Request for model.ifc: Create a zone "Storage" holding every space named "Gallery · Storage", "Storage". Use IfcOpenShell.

First a look at what the model holds.

```python
import ifcopenshell

model = ifcopenshell.open("model.ifc")
print(model.schema)
seen = {}
for space in model.by_type("IfcSpace"):
    seen[space.Name] = seen.get(space.Name, 0) + 1
for name, count in sorted(seen.items(), key=str):
    print(count, "x", name)
print("zones:", [z.Name for z in model.by_type("IfcZone")][:20])
```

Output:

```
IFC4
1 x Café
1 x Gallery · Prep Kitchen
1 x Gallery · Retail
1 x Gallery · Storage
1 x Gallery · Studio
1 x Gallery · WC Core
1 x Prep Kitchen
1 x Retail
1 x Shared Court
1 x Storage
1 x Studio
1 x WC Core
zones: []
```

```python
import ifcopenshell
import ifcopenshell.api.group
import ifcopenshell.api.root

model = ifcopenshell.open("model.ifc")

names = {"Gallery · Storage", "Storage"}
spaces = [s for s in model.by_type("IfcSpace") if s.Name in names]

zone = ifcopenshell.api.root.create_entity(model, ifc_class="IfcZone", name="Storage")
ifcopenshell.api.group.assign_group(model, products=spaces, group=zone)
print(len(spaces), "spaces in", zone.Name)

model.write("model_edited.ifc")
```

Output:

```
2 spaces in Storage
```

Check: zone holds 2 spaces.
